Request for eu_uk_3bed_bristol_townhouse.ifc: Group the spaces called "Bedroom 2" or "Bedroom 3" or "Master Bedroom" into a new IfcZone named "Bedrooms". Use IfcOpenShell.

First a look at what the model holds.

```python
import ifcopenshell

model = ifcopenshell.open("eu_uk_3bed_bristol_townhouse.ifc")
print(model.schema)
seen = {}
for space in model.by_type("IfcSpace"):
    seen[space.LongName] = seen.get(space.LongName, 0) + 1
for name, count in sorted(seen.items(), key=str):
    print(count, "x", name)
print("zones:", [z.Name for z in model.by_type("IfcZone")][:20])
```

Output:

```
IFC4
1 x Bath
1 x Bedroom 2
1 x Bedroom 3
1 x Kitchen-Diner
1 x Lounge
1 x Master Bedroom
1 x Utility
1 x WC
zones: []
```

```python
import ifcopenshell
import ifcopenshell.api.group
import ifcopenshell.api.root

model = ifcopenshell.open("eu_uk_3bed_bristol_townhouse.ifc")

names = {"Bedroom 2", "Bedroom 3", "Master Bedroom"}
spaces = [s for s in model.by_type("IfcSpace") if s.LongName in names]

zone = ifcopenshell.api.root.create_entity(model, ifc_class="IfcZone", name="Bedrooms")
ifcopenshell.api.group.assign_group(model, products=spaces, group=zone)
print(len(spaces), "spaces in", zone.Name)

model.write("eu_uk_3bed_bristol_townhouse_rev.ifc")
```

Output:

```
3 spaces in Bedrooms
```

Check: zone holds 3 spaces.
